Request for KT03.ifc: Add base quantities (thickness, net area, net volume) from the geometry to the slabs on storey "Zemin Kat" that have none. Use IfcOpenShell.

First a look at what the model holds.

```python
import ifcopenshell
import ifcopenshell.util.element
import ifcopenshell.util.unit

model = ifcopenshell.open("KT03.ifc")
print(model.schema)
for unit_type in ("LENGTHUNIT", "AREAUNIT", "VOLUMEUNIT"):
    print(unit_type, ifcopenshell.util.unit.calculate_unit_scale(model, unit_type))
storey = next(s for s in model.by_type("IfcBuildingStorey") if s.Name == "Zemin Kat")
slabs = [e for e in ifcopenshell.util.element.get_decomposition(storey) if e.is_a("IfcSlab")]
for e in sorted(slabs, key=lambda e: e.id()):
    print(e.id(), e.is_a(), e.Name, list(ifcopenshell.util.element.get_psets(e, qtos_only=True)), sep=" | ")
```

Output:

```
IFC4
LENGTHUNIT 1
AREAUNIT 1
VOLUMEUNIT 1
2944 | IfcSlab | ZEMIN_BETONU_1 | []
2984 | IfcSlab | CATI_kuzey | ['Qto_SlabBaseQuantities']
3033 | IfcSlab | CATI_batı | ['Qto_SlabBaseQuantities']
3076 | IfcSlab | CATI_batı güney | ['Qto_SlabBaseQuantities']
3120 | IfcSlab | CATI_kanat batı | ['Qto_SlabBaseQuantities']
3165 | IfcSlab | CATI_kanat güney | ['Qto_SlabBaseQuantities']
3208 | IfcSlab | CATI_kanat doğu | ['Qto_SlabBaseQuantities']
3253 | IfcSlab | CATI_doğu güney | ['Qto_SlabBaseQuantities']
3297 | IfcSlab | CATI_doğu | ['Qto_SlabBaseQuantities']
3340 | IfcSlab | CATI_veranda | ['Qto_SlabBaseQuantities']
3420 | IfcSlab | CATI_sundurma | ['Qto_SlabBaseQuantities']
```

```python
import ifcopenshell
import ifcopenshell.api.pset
import ifcopenshell.geom
import ifcopenshell.util.element
import ifcopenshell.util.shape
import ifcopenshell.util.unit

model = ifcopenshell.open("KT03.ifc")
unit_scale = ifcopenshell.util.unit.calculate_unit_scale(model)
area_scale = ifcopenshell.util.unit.calculate_unit_scale(model, "AREAUNIT")
volume_scale = ifcopenshell.util.unit.calculate_unit_scale(model, "VOLUMEUNIT")
settings = ifcopenshell.geom.settings()

storey = next(s for s in model.by_type("IfcBuildingStorey") if s.Name == "Zemin Kat")
slabs = [e for e in ifcopenshell.util.element.get_decomposition(storey) if e.is_a("IfcSlab")]

for e in sorted(slabs, key=lambda e: e.id()):
    if ifcopenshell.util.element.get_psets(e, qtos_only=True, should_inherit=False):
        continue
    # Geometry comes back in metres, in the element's own axes.
    shape = ifcopenshell.geom.create_shape(settings, e)
    values = {
        "Width": ifcopenshell.util.shape.get_z(shape.geometry) / unit_scale,
        "NetArea": ifcopenshell.util.shape.get_footprint_area(shape.geometry) / area_scale,
        "NetVolume": ifcopenshell.util.shape.get_volume(shape.geometry) / volume_scale,
    }
    qto = ifcopenshell.api.pset.add_qto(model, product=e, name="Qto_SlabBaseQuantities")
    ifcopenshell.api.pset.edit_qto(model, qto=qto, properties=values)
    print(e.id(), {k: round(v, 3) for k, v in values.items()})

model.write("KT03_edited.ifc")
```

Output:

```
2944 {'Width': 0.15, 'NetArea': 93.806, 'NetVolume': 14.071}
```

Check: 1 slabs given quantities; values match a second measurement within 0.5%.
